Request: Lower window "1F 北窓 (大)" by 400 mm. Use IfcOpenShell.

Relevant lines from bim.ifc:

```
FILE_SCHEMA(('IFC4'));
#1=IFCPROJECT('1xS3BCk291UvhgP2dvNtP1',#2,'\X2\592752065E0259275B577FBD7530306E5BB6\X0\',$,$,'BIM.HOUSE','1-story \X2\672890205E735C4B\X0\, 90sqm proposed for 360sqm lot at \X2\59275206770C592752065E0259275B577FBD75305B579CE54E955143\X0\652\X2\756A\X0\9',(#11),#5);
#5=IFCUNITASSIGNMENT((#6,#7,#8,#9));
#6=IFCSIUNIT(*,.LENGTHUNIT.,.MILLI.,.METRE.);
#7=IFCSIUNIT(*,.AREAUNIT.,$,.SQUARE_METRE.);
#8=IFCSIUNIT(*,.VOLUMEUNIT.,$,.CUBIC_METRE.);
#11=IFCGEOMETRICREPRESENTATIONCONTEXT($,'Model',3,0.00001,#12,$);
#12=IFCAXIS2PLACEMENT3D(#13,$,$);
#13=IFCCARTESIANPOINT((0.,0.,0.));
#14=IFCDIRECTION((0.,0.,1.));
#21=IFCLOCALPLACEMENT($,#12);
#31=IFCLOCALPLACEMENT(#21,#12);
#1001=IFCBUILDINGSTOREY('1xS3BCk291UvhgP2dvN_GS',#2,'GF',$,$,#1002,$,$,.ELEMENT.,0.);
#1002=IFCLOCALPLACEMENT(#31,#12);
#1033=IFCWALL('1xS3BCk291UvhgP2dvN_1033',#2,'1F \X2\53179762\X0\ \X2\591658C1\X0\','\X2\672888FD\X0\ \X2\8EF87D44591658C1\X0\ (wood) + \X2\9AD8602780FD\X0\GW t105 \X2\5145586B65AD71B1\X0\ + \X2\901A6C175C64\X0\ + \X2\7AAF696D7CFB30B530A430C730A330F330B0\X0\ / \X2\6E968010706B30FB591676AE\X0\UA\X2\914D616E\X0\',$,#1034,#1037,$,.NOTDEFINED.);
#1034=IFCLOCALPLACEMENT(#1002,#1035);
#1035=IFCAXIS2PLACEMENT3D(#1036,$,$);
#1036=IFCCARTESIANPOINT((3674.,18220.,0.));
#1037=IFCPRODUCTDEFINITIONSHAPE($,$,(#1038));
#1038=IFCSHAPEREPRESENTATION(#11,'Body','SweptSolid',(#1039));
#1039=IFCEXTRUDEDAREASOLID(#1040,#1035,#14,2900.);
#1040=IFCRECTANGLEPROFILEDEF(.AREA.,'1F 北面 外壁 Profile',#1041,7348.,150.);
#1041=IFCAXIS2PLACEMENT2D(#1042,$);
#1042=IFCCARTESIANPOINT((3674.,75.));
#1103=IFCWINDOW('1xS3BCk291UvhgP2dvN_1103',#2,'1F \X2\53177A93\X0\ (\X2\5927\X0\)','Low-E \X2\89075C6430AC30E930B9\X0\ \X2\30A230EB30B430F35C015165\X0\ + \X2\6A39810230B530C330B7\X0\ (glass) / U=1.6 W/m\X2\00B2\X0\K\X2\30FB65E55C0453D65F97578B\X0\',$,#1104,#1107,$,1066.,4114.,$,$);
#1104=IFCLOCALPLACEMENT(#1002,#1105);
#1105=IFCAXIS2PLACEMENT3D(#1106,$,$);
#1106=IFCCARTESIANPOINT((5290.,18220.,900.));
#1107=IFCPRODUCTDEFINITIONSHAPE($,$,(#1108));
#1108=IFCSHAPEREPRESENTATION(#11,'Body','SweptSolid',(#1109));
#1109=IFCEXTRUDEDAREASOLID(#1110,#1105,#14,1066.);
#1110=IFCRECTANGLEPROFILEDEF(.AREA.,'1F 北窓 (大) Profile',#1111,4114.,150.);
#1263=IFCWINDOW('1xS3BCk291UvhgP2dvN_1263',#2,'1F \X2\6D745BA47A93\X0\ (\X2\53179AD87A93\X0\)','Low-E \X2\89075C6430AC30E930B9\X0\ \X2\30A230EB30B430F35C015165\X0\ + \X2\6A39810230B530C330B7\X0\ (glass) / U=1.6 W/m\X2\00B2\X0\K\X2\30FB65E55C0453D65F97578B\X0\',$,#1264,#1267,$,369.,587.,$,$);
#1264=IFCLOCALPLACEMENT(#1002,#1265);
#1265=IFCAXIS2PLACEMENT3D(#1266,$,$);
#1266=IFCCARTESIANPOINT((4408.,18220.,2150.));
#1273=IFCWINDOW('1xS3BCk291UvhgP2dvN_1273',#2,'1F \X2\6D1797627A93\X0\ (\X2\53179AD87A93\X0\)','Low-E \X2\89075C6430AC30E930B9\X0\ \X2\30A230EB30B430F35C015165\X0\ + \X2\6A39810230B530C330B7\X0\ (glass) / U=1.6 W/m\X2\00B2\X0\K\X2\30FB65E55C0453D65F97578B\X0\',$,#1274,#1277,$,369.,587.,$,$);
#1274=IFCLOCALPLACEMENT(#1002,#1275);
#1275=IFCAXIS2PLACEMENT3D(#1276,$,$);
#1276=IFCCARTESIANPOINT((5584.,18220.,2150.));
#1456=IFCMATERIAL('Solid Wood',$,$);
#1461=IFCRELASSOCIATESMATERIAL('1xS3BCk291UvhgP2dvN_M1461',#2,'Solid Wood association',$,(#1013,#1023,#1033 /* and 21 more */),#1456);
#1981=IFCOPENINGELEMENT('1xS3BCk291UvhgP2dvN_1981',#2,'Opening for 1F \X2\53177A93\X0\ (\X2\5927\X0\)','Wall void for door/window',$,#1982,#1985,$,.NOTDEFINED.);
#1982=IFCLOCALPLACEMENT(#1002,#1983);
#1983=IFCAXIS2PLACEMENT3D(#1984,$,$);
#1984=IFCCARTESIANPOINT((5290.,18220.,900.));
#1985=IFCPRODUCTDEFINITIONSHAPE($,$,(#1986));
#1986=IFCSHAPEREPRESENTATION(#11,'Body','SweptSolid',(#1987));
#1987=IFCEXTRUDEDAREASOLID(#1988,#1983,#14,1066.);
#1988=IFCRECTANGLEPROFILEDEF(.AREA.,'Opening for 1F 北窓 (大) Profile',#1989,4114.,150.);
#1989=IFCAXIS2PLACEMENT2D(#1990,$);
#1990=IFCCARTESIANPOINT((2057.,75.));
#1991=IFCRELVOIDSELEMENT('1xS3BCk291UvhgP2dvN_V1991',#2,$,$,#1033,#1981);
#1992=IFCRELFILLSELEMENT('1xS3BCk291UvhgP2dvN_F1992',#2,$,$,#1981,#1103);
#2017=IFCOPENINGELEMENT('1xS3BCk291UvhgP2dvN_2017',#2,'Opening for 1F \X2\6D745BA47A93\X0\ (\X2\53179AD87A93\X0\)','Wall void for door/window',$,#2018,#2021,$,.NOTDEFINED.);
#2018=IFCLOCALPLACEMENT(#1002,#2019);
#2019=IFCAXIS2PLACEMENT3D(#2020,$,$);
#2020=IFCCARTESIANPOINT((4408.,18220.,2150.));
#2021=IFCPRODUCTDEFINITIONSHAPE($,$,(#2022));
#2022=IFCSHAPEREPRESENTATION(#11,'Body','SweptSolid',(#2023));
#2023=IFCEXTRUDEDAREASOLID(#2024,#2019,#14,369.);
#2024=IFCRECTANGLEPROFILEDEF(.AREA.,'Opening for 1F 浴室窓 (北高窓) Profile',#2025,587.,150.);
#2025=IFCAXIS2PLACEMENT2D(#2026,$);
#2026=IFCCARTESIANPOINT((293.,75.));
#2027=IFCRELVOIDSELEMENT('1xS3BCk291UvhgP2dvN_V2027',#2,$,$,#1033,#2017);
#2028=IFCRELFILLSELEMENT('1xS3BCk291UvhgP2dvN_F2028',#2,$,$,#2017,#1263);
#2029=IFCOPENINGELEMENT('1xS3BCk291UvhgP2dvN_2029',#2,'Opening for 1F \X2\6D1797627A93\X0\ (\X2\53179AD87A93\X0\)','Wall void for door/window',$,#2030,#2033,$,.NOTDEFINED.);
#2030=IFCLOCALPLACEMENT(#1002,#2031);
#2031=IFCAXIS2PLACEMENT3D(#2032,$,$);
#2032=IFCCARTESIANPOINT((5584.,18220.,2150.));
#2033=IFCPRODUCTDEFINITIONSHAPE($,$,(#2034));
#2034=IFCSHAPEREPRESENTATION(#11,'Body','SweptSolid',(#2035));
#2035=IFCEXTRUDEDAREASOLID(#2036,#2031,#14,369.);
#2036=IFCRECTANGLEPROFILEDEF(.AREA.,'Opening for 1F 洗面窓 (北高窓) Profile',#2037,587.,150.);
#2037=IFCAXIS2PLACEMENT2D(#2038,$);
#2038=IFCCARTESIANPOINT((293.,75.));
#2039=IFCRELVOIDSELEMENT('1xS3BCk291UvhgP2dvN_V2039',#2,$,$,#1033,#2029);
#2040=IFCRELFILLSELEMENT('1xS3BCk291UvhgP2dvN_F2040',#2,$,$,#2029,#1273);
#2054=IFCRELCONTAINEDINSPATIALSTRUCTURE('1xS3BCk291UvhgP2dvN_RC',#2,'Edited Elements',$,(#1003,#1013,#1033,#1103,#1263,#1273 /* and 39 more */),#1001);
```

```python
import numpy as np
import ifcopenshell
import ifcopenshell.api.geometry
import ifcopenshell.util.placement
import ifcopenshell.util.unit

model = ifcopenshell.open("bim.ifc")
unit_scale = ifcopenshell.util.unit.calculate_unit_scale(model)

window = model.by_guid("1xS3BCk291UvhgP2dvN_1103")
opening = window.FillsVoids[0].RelatingOpeningElement
dz = -0.4 / unit_scale

shift = np.array([0.0, 0.0, dz])
# The window is not placed relative to its opening, so move both.
for product in (opening, window):
    matrix = ifcopenshell.util.placement.get_local_placement(product.ObjectPlacement)
    matrix[:3, 3] += shift
    ifcopenshell.api.geometry.edit_object_placement(model, product=product, matrix=matrix, is_si=False)

print(f"moved by {dz * unit_scale:+.3f} m")

model.write("bim_rev.ifc")
```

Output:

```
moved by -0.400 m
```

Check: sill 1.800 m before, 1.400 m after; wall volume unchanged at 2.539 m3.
